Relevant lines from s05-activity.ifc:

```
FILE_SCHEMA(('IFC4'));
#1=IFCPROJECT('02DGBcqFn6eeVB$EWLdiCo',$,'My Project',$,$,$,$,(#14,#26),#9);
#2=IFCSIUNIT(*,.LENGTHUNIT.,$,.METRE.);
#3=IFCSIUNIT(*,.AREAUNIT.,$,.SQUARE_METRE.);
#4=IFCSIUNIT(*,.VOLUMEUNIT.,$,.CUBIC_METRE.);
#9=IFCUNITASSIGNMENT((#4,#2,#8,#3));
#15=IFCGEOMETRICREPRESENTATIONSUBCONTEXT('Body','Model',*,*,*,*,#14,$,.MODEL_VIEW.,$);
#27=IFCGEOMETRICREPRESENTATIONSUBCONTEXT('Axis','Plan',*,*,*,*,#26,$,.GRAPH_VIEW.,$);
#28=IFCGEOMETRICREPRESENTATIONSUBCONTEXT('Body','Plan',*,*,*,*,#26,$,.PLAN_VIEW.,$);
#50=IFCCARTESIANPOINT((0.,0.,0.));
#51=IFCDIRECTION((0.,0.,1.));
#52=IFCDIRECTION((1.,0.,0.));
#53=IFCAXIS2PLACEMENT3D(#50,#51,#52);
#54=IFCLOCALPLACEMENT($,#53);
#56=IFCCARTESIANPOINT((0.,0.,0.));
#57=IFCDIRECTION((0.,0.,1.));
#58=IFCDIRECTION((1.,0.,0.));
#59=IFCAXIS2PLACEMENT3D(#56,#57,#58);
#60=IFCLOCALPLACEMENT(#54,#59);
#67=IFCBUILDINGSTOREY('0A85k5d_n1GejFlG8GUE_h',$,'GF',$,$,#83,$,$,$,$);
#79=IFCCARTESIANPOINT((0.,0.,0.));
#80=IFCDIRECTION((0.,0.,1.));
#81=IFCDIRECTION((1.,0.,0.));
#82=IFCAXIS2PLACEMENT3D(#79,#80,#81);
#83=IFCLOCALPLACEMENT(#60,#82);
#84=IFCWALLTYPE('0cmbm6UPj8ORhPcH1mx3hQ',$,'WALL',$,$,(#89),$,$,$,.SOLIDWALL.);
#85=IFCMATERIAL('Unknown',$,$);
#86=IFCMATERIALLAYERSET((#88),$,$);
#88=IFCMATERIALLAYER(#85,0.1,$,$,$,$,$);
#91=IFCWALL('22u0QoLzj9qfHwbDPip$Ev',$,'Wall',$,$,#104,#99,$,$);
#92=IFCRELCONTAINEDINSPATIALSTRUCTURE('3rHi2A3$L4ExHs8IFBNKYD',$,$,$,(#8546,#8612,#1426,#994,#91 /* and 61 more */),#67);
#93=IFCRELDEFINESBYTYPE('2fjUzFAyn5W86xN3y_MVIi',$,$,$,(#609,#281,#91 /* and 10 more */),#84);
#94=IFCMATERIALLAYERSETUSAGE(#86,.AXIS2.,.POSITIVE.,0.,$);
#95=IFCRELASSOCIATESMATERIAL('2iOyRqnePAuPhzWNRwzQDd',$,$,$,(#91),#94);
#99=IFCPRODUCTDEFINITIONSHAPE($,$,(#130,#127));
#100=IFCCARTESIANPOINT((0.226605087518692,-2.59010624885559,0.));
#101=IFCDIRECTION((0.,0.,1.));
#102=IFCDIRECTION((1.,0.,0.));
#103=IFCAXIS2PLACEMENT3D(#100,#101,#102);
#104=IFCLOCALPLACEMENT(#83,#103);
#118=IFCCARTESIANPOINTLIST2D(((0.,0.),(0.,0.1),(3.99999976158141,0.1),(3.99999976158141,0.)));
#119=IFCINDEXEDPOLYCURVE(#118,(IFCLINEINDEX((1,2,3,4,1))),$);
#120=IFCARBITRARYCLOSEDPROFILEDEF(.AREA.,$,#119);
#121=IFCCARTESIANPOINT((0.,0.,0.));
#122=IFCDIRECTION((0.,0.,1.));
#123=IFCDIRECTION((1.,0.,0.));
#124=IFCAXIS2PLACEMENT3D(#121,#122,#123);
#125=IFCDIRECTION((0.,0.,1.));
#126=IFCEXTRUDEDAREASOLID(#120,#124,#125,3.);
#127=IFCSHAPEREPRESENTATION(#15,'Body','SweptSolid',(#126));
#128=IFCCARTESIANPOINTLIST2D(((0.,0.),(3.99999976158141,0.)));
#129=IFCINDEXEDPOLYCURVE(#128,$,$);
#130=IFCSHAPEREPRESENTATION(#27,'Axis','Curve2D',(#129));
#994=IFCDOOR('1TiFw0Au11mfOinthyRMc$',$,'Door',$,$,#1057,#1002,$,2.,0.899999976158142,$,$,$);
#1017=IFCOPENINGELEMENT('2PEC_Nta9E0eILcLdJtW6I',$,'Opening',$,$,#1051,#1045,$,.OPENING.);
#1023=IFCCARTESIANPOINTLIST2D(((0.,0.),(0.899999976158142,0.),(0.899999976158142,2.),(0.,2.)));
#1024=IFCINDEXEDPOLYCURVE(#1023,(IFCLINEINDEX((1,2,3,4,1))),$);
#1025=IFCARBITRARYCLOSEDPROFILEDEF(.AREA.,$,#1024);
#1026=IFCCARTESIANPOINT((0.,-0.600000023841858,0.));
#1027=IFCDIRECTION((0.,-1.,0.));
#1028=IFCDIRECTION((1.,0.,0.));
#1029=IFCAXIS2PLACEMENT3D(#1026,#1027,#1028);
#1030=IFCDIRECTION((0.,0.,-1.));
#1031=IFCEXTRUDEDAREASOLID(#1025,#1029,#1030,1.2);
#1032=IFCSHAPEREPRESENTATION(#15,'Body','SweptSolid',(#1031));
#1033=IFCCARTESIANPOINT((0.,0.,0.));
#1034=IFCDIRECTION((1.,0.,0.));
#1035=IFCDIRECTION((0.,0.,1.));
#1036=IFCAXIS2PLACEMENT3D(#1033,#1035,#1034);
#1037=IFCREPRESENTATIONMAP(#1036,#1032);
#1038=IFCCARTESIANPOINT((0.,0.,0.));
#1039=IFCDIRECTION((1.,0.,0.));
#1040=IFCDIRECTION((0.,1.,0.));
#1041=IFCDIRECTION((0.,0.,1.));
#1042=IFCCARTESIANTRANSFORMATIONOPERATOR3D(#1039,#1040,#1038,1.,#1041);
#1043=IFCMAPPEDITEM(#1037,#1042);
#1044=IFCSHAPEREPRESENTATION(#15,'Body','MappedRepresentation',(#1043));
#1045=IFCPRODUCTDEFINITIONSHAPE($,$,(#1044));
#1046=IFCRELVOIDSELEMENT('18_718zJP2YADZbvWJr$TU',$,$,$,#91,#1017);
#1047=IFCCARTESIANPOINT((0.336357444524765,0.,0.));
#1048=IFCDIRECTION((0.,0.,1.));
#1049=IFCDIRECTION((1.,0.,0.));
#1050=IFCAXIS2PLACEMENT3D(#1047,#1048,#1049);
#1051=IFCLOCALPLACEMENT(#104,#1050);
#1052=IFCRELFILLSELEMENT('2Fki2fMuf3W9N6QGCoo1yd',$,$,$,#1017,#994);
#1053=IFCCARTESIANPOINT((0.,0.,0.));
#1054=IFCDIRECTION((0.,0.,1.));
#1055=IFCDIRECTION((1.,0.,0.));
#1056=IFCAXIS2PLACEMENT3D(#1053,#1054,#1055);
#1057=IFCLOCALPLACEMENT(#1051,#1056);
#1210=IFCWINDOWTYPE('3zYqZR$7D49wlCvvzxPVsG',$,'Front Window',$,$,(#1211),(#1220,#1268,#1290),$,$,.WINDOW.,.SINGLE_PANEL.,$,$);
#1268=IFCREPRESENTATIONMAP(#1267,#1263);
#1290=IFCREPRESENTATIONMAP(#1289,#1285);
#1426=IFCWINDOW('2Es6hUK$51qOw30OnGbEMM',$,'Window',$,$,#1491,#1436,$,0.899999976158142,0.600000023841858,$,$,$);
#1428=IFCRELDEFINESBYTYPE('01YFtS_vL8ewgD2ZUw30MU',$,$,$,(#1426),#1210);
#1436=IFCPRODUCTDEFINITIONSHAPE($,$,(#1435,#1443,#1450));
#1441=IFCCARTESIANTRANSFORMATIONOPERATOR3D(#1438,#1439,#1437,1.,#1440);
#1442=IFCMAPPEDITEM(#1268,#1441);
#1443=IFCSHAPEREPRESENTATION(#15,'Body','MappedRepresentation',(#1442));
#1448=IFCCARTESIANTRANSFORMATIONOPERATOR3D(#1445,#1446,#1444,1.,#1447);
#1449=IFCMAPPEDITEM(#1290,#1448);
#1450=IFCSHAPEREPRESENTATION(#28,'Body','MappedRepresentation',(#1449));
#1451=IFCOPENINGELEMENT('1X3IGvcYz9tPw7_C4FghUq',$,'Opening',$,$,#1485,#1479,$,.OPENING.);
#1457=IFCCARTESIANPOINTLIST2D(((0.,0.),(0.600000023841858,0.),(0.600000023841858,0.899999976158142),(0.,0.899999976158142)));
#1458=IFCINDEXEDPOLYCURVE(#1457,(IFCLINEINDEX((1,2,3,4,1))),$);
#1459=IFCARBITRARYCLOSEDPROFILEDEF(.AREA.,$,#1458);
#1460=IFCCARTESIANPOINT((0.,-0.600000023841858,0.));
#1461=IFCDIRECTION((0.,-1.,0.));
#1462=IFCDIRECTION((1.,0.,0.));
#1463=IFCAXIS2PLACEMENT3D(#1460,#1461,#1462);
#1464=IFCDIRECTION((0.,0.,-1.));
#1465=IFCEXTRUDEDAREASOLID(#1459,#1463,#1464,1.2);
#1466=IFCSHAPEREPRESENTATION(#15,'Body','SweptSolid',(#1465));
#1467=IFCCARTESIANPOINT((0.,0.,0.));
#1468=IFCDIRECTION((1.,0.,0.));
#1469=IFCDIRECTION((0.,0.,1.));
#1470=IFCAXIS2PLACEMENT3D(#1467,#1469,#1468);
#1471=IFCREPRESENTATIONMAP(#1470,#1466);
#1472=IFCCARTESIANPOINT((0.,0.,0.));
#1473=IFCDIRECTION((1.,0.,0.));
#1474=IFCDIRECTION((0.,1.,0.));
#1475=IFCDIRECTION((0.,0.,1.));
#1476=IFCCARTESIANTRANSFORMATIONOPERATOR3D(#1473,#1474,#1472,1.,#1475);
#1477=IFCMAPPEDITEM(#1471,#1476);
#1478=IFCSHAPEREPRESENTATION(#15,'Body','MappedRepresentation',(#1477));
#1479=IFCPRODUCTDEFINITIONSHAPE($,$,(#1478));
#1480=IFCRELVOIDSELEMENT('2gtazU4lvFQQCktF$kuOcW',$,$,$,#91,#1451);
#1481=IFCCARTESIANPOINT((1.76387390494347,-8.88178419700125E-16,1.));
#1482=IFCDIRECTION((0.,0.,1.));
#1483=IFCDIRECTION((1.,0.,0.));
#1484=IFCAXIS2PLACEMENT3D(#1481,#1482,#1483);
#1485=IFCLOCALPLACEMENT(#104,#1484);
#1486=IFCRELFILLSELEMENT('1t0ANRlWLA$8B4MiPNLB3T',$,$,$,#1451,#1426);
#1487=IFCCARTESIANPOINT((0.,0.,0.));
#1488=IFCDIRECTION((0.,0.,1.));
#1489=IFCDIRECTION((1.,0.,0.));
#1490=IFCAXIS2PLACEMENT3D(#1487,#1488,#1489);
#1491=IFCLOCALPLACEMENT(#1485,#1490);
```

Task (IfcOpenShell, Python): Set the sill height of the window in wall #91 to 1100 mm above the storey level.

```python
import numpy as np
import ifcopenshell
import ifcopenshell.api.geometry
import ifcopenshell.geom
import ifcopenshell.util.element
import ifcopenshell.util.placement
import ifcopenshell.util.shape
import ifcopenshell.util.unit

model = ifcopenshell.open("s05-activity.ifc")
unit_scale = ifcopenshell.util.unit.calculate_unit_scale(model)

window = model.by_guid("2Es6hUK$51qOw30OnGbEMM")
opening = window.FillsVoids[0].RelatingOpeningElement
storey = ifcopenshell.util.element.get_container(window, ifc_class="IfcBuildingStorey")
level = ifcopenshell.util.placement.get_local_placement(storey.ObjectPlacement)[2, 3]

# The opening's origin need not be at the sill, so measure its lowest point.
shape = ifcopenshell.geom.create_shape(ifcopenshell.geom.settings(), opening)
bottom = ifcopenshell.util.shape.get_shape_bottom_elevation(shape, shape.geometry) / unit_scale
dz = level + 1.1 / unit_scale - bottom

shift = np.array([0.0, 0.0, dz])
# The window is placed relative to its opening, so it follows when the opening moves.
matrix = ifcopenshell.util.placement.get_local_placement(opening.ObjectPlacement)
matrix[:3, 3] += shift
ifcopenshell.api.geometry.edit_object_placement(
    model, product=opening, matrix=matrix, is_si=False, should_transform_children=True
)

print(f"moved by {dz * unit_scale:+.3f} m")

model.write("s05-activity_edited.ifc")
```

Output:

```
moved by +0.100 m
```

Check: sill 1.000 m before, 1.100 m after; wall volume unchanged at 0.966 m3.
